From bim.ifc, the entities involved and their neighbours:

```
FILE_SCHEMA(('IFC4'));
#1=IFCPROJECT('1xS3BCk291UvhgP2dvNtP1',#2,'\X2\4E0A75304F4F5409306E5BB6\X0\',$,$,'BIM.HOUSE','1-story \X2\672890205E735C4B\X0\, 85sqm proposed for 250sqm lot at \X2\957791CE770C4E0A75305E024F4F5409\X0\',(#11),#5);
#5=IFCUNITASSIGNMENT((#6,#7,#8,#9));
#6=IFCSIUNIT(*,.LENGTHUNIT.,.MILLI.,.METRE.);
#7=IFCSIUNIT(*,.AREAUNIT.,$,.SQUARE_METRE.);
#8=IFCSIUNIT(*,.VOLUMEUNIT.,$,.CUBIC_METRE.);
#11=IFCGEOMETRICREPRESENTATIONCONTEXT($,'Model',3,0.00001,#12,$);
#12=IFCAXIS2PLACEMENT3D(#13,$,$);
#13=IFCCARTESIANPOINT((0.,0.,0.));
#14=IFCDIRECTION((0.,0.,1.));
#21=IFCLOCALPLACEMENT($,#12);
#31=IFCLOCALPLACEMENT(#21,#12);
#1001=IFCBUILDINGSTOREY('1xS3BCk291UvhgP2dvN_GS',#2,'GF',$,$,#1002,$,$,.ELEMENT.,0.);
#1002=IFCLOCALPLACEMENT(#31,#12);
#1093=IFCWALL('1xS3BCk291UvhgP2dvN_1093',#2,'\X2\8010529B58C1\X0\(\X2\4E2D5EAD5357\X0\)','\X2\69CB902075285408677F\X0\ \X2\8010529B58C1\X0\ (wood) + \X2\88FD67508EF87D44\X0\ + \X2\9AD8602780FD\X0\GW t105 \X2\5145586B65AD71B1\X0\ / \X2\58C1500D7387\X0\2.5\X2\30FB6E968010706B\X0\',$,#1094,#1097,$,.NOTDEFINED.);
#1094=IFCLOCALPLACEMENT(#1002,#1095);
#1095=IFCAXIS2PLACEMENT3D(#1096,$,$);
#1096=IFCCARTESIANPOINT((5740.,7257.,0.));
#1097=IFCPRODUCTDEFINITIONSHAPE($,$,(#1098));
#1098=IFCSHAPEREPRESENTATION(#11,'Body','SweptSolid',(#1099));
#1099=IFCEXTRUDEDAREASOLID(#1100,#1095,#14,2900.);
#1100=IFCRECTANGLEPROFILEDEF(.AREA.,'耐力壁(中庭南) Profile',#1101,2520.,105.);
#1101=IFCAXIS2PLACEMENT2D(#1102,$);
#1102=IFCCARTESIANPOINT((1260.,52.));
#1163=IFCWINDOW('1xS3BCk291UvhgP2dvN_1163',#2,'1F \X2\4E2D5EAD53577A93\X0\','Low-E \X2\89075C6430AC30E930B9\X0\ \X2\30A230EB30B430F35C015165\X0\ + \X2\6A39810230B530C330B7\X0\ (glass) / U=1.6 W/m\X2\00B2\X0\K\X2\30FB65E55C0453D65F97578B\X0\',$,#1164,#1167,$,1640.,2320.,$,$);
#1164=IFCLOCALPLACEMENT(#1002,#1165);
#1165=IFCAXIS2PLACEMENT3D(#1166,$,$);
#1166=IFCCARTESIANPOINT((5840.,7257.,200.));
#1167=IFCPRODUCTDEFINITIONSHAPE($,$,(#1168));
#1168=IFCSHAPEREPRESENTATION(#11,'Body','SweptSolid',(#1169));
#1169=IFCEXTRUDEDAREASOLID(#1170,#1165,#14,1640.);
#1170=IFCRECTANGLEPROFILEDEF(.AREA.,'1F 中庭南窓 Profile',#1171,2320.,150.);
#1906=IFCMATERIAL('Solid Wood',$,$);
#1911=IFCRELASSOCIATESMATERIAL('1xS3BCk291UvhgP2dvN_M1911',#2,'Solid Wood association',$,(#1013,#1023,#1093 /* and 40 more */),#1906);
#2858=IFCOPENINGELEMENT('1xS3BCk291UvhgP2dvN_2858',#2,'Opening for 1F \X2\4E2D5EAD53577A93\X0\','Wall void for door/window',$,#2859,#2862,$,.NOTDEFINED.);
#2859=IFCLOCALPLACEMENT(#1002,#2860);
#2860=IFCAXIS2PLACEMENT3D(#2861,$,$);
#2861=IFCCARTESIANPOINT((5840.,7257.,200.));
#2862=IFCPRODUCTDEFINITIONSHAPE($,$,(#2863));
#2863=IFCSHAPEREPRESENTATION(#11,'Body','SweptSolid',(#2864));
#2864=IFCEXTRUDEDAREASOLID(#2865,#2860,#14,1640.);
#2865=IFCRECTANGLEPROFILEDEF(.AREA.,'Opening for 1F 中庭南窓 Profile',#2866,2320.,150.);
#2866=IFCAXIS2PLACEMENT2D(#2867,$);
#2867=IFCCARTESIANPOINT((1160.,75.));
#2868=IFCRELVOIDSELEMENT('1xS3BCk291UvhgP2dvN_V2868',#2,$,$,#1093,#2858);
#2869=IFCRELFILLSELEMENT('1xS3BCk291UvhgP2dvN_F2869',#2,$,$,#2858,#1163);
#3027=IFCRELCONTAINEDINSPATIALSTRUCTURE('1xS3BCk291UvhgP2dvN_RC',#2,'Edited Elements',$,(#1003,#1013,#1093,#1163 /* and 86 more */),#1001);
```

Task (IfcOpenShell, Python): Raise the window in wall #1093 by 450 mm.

```python
import numpy as np
import ifcopenshell
import ifcopenshell.api.geometry
import ifcopenshell.util.placement
import ifcopenshell.util.unit

model = ifcopenshell.open("bim.ifc")
unit_scale = ifcopenshell.util.unit.calculate_unit_scale(model)

window = model.by_guid("1xS3BCk291UvhgP2dvN_1163")
opening = window.FillsVoids[0].RelatingOpeningElement
dz = 0.45 / unit_scale

shift = np.array([0.0, 0.0, dz])
# The window is not placed relative to its opening, so move both.
for product in (opening, window):
    matrix = ifcopenshell.util.placement.get_local_placement(product.ObjectPlacement)
    matrix[:3, 3] += shift
    ifcopenshell.api.geometry.edit_object_placement(model, product=product, matrix=matrix, is_si=False)

print(f"moved by {dz * unit_scale:+.3f} m")

model.write("bim-out.ifc")
```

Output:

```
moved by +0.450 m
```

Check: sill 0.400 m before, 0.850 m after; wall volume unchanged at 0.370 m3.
